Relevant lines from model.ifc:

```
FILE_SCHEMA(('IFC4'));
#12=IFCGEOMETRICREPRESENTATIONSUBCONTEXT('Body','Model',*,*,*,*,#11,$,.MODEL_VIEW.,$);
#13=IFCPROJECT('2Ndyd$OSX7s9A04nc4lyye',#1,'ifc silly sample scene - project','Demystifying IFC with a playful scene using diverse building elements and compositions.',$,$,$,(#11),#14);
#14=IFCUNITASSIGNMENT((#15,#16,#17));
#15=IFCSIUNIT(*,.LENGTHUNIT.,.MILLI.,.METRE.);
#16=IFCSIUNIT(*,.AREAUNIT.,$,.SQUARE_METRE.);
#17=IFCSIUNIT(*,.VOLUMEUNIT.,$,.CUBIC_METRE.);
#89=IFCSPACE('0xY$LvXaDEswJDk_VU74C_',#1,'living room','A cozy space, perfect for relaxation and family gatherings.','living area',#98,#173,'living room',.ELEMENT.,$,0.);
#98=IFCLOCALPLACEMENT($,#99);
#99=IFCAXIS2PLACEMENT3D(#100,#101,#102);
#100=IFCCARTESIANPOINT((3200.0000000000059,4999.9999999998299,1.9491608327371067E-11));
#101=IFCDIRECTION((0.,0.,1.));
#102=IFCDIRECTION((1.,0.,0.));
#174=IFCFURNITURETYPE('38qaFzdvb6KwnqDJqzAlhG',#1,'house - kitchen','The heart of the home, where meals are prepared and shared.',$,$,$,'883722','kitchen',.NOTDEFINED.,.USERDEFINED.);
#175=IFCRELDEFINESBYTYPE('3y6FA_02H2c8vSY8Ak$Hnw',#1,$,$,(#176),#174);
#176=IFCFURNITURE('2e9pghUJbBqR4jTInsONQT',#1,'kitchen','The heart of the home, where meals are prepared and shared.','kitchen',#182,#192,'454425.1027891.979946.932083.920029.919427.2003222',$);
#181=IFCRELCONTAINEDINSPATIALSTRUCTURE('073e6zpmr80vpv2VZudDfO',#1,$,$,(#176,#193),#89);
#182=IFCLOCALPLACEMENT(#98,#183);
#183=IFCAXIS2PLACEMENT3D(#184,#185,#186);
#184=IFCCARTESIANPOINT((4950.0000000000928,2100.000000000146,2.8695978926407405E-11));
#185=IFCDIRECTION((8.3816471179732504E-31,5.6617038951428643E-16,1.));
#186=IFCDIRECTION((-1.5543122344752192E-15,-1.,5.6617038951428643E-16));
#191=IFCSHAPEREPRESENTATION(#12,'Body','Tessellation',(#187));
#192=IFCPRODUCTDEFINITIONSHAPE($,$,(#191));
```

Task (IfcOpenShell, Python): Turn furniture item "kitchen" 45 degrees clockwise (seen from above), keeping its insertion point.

```python
import ifcopenshell
import ifcopenshell.api.geometry
import ifcopenshell.util.placement

model = ifcopenshell.open("model.ifc")

item = model.by_guid("2e9pghUJbBqR4jTInsONQT")
matrix = ifcopenshell.util.placement.get_local_placement(item.ObjectPlacement)
matrix = matrix @ ifcopenshell.util.placement.rotation(-45, "Z")
ifcopenshell.api.geometry.edit_object_placement(model, product=item, matrix=matrix, is_si=False)

print(ifcopenshell.util.placement.get_local_placement(item.ObjectPlacement).round(3) + 0.0)

model.write("model_rev.ifc")
```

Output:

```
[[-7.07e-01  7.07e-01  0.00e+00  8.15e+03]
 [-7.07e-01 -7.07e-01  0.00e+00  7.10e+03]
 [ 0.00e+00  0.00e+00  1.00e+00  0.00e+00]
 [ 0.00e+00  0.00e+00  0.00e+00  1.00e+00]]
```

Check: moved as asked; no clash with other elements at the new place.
